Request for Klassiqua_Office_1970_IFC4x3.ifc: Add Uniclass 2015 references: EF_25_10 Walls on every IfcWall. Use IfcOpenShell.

First a look at what the model holds.

```python
import ifcopenshell

model = ifcopenshell.open("Klassiqua_Office_1970_IFC4x3.ifc")
print(model.schema)
print("classifications:", [c.Name for c in model.by_type("IfcClassification")])
for ifc_class in ("IfcDoor", "IfcRoof", "IfcStair", "IfcWall", "IfcWindow"):
    print(ifc_class, len(model.by_type(ifc_class)))
```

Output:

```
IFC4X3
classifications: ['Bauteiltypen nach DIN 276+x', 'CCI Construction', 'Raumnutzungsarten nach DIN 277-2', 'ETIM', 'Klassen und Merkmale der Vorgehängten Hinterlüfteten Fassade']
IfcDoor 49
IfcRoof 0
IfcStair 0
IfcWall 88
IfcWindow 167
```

```python
import ifcopenshell
import ifcopenshell.api.classification

model = ifcopenshell.open("Klassiqua_Office_1970_IFC4x3.ifc")

system = ifcopenshell.api.classification.add_classification(model, classification="Uniclass 2015")

codes = {
    "IfcWall": ("EF_25_10", "Walls"),
}
for ifc_class, (code, name) in codes.items():
    products = model.by_type(ifc_class)
    ifcopenshell.api.classification.add_reference(
        model, products=products, classification=system, identification=code, name=name
    )
    print(code, len(products))

model.write("Klassiqua_Office_1970_IFC4x3_rev.ifc")
```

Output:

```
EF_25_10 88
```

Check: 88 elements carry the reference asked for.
